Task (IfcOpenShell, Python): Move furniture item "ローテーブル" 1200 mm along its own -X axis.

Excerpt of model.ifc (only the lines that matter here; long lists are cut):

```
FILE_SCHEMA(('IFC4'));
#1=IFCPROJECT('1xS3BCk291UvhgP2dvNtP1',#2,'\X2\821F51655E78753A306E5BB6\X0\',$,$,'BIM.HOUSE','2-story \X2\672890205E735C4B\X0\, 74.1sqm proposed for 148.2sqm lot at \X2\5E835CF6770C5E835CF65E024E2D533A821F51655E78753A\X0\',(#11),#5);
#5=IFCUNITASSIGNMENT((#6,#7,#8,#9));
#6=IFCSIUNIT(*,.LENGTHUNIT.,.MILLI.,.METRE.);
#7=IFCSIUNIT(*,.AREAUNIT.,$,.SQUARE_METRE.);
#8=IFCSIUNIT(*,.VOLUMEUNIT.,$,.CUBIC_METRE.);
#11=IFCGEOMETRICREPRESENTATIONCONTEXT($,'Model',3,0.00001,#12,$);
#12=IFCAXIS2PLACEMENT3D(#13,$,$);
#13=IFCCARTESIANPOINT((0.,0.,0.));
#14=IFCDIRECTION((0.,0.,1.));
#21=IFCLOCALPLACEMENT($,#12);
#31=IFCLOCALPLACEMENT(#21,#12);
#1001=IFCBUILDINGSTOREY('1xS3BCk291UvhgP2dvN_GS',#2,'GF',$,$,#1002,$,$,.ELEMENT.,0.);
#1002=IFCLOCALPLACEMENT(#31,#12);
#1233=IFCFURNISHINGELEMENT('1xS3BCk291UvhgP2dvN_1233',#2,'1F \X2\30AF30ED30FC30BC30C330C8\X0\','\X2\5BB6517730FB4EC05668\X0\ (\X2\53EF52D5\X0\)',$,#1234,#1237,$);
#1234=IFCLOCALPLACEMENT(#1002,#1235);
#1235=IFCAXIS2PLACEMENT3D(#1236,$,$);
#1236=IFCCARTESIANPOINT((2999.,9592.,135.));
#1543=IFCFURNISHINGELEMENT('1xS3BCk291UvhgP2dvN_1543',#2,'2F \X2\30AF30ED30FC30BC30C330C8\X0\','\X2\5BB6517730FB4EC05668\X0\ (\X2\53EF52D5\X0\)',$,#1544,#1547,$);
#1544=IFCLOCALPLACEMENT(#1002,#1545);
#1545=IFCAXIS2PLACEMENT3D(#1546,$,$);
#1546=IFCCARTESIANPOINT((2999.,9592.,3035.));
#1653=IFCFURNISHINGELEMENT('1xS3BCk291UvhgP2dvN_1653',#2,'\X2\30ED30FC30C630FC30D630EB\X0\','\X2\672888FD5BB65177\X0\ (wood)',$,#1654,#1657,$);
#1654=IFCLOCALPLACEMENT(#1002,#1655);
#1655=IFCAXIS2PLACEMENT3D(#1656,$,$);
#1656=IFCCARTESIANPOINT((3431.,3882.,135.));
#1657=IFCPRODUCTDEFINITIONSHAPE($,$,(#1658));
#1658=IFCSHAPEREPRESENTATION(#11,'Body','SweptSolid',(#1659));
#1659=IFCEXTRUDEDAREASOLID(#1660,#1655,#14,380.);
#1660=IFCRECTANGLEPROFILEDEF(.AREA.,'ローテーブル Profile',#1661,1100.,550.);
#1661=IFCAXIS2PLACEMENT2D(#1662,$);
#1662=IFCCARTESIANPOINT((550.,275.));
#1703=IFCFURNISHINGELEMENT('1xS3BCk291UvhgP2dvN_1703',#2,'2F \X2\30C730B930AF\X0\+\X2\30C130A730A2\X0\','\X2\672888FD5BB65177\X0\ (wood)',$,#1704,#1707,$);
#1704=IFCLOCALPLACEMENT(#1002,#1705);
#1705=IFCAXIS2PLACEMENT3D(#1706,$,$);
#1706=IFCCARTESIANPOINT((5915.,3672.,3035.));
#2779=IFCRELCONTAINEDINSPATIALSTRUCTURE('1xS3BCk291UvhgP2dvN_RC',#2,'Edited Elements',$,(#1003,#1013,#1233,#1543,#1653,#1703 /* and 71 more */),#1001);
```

```python
import ifcopenshell
import ifcopenshell.api.geometry
import ifcopenshell.util.placement

model = ifcopenshell.open("model.ifc")

item = model.by_id(1653)
matrix = ifcopenshell.util.placement.get_local_placement(item.ObjectPlacement)
matrix[:3, 3] -= matrix[:3, 0] * 1200.0
ifcopenshell.api.geometry.edit_object_placement(model, product=item, matrix=matrix, is_si=False)

print(ifcopenshell.util.placement.get_local_placement(item.ObjectPlacement).round(3) + 0.0)

model.write("model-out.ifc")
```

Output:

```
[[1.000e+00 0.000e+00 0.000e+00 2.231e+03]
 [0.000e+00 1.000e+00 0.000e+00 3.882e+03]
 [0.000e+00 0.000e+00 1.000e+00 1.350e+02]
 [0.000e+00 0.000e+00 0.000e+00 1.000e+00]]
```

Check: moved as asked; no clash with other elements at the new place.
